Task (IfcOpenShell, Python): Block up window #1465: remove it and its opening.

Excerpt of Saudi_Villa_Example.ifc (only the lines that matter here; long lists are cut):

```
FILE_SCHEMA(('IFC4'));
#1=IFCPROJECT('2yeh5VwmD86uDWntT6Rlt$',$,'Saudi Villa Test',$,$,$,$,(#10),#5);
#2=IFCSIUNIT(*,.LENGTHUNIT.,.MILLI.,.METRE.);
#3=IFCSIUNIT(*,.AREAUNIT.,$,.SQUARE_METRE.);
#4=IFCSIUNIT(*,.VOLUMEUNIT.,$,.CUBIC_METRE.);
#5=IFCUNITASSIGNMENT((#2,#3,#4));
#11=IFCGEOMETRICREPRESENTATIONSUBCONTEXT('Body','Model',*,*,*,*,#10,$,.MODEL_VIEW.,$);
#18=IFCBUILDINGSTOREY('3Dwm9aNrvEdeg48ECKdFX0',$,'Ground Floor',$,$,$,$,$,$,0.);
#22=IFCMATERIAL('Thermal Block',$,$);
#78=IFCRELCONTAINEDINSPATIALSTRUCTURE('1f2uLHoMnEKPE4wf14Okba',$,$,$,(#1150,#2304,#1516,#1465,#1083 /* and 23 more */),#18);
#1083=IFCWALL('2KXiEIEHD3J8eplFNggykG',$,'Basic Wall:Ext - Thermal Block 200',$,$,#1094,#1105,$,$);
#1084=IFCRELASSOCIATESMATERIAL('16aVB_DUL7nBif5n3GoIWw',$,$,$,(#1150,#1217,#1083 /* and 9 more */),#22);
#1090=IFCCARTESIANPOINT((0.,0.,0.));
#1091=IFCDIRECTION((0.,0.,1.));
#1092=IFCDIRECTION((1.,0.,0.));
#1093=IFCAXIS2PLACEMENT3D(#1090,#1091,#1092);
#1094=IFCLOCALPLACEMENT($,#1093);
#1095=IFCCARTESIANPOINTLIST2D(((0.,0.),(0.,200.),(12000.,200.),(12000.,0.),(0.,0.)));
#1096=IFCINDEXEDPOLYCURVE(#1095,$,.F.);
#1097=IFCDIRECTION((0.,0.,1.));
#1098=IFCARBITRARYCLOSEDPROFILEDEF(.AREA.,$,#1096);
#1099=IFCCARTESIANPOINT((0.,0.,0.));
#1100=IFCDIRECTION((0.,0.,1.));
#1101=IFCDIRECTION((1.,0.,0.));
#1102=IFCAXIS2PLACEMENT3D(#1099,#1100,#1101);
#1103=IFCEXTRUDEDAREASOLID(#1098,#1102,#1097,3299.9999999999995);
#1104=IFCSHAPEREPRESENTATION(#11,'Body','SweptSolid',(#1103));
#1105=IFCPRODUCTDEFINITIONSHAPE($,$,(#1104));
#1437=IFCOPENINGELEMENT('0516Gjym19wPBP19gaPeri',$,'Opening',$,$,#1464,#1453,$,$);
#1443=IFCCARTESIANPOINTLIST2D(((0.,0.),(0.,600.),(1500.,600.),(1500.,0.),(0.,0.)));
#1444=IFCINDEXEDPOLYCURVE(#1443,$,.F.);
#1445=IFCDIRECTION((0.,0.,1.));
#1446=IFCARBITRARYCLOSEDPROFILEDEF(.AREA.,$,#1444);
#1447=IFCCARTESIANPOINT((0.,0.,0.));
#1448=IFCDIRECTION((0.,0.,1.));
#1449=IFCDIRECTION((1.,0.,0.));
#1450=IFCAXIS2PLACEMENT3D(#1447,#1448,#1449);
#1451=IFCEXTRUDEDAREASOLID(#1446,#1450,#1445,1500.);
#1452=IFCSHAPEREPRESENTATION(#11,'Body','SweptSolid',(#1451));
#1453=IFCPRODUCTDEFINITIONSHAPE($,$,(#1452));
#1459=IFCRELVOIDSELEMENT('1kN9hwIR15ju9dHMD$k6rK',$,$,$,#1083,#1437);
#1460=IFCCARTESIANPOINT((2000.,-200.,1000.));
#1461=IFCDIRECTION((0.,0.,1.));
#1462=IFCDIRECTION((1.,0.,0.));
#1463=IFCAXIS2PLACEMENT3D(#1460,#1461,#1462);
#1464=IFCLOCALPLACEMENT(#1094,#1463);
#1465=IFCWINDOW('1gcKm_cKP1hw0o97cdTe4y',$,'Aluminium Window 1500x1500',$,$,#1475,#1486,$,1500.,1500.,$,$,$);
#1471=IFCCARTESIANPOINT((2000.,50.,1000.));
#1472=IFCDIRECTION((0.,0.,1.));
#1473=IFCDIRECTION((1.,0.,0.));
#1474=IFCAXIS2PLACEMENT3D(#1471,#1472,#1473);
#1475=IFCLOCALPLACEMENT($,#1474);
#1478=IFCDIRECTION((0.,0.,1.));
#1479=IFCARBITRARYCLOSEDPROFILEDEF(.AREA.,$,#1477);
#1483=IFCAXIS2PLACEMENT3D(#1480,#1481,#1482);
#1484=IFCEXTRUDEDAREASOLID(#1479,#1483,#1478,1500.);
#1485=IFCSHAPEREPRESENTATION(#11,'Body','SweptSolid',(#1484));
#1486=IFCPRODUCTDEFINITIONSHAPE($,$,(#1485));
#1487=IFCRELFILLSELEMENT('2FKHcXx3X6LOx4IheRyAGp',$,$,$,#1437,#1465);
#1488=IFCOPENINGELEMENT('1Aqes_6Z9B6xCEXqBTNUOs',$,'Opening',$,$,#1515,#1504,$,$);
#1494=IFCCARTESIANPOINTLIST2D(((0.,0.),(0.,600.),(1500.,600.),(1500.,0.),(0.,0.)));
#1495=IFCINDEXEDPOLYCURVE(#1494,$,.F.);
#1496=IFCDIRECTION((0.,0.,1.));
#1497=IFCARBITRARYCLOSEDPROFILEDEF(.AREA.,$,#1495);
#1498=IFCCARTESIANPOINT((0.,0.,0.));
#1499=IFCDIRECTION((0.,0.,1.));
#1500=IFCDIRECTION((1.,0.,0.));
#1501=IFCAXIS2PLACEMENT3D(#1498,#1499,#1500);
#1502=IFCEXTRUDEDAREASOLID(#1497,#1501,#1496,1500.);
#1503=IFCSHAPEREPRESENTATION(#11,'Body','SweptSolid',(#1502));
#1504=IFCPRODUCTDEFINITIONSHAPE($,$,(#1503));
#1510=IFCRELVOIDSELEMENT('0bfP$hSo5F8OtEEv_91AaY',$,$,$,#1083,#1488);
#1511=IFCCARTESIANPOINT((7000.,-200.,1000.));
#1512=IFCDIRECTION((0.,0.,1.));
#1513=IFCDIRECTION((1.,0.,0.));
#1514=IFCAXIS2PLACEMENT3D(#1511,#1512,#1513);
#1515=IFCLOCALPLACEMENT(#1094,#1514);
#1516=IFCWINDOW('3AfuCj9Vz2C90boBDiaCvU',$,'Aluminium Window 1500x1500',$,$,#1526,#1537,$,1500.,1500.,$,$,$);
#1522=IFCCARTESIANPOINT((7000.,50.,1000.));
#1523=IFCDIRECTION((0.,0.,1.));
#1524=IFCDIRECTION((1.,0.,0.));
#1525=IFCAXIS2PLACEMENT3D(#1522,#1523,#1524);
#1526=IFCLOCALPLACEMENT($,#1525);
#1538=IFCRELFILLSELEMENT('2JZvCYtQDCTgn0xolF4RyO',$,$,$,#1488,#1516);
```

```python
import ifcopenshell
import ifcopenshell.api.feature
import ifcopenshell.api.root
import ifcopenshell.geom
import ifcopenshell.util.shape

model = ifcopenshell.open("Saudi_Villa_Example.ifc")
settings = ifcopenshell.geom.settings()


def volume(element):
    """Net volume in cubic metres, openings subtracted."""
    shape = ifcopenshell.geom.create_shape(settings, element)
    return ifcopenshell.util.shape.get_volume(shape.geometry)


window = model.by_guid("1gcKm_cKP1hw0o97cdTe4y")
opening = window.FillsVoids[0].RelatingOpeningElement
wall = opening.VoidsElements[0].RelatingBuildingElement
before = volume(wall)

ifcopenshell.api.root.remove_product(model, product=window)
ifcopenshell.api.feature.remove_feature(model, feature=opening)

after = volume(wall)

print(f"wall volume {before:.3f} -> {after:.3f} m3")

model.write("Saudi_Villa_Example_v2.ifc")
```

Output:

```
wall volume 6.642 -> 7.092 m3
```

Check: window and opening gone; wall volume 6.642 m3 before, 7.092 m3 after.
